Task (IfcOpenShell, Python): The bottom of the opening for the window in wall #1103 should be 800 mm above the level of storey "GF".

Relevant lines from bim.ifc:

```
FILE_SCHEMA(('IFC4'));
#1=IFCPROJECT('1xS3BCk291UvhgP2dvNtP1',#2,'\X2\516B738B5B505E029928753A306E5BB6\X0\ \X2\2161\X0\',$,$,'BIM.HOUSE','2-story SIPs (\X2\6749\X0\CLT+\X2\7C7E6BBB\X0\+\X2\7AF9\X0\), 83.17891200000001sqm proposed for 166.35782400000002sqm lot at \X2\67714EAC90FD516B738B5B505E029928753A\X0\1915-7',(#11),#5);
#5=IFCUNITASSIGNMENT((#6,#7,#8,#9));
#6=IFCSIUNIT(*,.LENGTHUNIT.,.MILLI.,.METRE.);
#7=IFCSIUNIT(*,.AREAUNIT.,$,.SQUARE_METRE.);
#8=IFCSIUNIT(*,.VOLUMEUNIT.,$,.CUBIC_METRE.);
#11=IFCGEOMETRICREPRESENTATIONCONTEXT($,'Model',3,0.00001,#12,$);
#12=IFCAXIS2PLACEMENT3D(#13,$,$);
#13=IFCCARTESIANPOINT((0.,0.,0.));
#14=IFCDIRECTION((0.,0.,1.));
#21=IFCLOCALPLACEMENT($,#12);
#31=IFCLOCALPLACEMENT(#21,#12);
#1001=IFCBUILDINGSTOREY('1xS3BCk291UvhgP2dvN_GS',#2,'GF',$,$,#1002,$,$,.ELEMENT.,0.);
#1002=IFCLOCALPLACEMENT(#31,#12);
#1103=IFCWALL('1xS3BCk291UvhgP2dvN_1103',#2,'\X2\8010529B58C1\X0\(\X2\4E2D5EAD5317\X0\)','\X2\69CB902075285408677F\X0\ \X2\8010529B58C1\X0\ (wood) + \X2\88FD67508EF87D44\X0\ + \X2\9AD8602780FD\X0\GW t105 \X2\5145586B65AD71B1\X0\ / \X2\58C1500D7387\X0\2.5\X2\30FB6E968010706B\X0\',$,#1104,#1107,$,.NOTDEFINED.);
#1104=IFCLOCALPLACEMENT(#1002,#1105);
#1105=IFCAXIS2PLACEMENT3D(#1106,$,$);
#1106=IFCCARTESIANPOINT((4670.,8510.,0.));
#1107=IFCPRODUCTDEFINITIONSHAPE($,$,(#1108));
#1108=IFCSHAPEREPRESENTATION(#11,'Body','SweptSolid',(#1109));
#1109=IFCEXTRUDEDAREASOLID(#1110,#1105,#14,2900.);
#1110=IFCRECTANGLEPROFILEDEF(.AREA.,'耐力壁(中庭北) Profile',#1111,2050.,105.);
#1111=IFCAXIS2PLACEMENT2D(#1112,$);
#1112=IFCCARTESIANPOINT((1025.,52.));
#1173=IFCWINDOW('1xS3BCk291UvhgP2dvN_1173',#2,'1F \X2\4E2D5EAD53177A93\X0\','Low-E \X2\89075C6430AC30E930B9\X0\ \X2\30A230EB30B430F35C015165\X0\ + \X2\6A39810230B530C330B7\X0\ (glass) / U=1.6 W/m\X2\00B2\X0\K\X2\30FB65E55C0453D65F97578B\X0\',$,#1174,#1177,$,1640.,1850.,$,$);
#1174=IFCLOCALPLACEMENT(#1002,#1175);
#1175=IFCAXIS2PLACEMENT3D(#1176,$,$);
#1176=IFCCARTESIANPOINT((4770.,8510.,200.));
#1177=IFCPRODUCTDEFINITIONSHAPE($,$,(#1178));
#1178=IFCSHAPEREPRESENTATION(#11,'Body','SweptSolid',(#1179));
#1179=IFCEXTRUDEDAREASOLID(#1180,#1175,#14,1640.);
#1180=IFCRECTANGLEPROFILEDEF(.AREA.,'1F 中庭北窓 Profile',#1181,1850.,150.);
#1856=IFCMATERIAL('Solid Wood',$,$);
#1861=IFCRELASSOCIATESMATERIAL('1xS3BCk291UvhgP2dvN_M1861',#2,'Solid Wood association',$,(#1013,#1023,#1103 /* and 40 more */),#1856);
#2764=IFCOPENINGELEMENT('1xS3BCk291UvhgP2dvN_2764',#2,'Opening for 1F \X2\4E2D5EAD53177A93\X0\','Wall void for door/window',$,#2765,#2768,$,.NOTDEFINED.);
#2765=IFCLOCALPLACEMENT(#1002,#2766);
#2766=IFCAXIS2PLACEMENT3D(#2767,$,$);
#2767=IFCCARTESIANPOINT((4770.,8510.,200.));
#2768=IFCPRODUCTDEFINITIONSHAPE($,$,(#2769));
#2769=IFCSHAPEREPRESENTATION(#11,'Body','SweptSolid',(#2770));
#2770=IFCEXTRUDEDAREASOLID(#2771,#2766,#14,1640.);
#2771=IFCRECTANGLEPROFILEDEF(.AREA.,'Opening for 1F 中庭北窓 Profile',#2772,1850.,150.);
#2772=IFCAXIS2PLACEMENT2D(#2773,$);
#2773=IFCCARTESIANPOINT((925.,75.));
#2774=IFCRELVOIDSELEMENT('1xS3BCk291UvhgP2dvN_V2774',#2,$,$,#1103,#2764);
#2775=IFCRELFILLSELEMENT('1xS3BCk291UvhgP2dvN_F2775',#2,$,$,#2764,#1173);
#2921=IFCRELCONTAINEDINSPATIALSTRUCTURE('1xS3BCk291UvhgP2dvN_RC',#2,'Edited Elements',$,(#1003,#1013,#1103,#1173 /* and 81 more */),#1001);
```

```python
import numpy as np
import ifcopenshell
import ifcopenshell.api.geometry
import ifcopenshell.geom
import ifcopenshell.util.element
import ifcopenshell.util.placement
import ifcopenshell.util.shape
import ifcopenshell.util.unit

model = ifcopenshell.open("bim.ifc")
unit_scale = ifcopenshell.util.unit.calculate_unit_scale(model)

window = model.by_id(1173)
opening = window.FillsVoids[0].RelatingOpeningElement
storey = ifcopenshell.util.element.get_container(window, ifc_class="IfcBuildingStorey")
level = ifcopenshell.util.placement.get_local_placement(storey.ObjectPlacement)[2, 3]

# The opening's origin need not be at the sill, so measure its lowest point.
shape = ifcopenshell.geom.create_shape(ifcopenshell.geom.settings(), opening)
bottom = ifcopenshell.util.shape.get_shape_bottom_elevation(shape, shape.geometry) / unit_scale
dz = level + 0.8 / unit_scale - bottom

shift = np.array([0.0, 0.0, dz])
# The window is not placed relative to its opening, so move both.
for product in (opening, window):
    matrix = ifcopenshell.util.placement.get_local_placement(product.ObjectPlacement)
    matrix[:3, 3] += shift
    ifcopenshell.api.geometry.edit_object_placement(model, product=product, matrix=matrix, is_si=False)

print(f"moved by {dz * unit_scale:+.3f} m")

model.write("bim_rev.ifc")
```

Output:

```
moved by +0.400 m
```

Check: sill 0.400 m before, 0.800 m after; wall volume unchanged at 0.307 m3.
